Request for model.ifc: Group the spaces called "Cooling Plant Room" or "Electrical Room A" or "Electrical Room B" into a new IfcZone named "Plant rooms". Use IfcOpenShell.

First a look at what the model holds.

```python
import ifcopenshell

model = ifcopenshell.open("model.ifc")
print(model.schema)
seen = {}
for space in model.by_type("IfcSpace"):
    seen[space.LongName] = seen.get(space.LongName, 0) + 1
for name, count in sorted(seen.items(), key=str):
    print(count, "x", name)
print("zones:", [z.Name for z in model.by_type("IfcZone")][:20])
```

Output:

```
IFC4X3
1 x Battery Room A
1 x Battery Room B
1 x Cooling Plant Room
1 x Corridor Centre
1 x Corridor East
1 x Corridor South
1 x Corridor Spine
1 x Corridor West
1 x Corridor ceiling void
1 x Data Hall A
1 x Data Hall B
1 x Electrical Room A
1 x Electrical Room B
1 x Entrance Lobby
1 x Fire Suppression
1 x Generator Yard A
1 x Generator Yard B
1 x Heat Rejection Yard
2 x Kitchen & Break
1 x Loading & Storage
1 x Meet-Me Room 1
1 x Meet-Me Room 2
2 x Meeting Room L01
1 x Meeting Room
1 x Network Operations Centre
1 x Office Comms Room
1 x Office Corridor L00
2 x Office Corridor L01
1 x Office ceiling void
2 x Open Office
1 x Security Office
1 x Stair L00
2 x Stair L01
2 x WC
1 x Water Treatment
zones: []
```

```python
import ifcopenshell
import ifcopenshell.api.group
import ifcopenshell.api.root

model = ifcopenshell.open("model.ifc")

names = {"Cooling Plant Room", "Electrical Room A", "Electrical Room B"}
spaces = [s for s in model.by_type("IfcSpace") if s.LongName in names]

zone = ifcopenshell.api.root.create_entity(model, ifc_class="IfcZone", name="Plant rooms")
ifcopenshell.api.group.assign_group(model, products=spaces, group=zone)
print(len(spaces), "spaces in", zone.Name)

model.write("model-out.ifc")
```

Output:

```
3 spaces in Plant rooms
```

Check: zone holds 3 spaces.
